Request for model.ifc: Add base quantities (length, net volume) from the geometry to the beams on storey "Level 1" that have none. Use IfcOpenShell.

First a look at what the model holds.

```python
import ifcopenshell
import ifcopenshell.util.element
import ifcopenshell.util.unit

model = ifcopenshell.open("model.ifc")
print(model.schema)
for unit_type in ("LENGTHUNIT", "AREAUNIT", "VOLUMEUNIT"):
    print(unit_type, ifcopenshell.util.unit.calculate_unit_scale(model, unit_type))
storey = next(s for s in model.by_type("IfcBuildingStorey") if s.Name == "Level 1")
beams = [e for e in ifcopenshell.util.element.get_decomposition(storey) if e.is_a("IfcBeam")]
for e in sorted(beams, key=lambda e: e.id()):
    print(e.id(), e.is_a(), e.Name, list(ifcopenshell.util.element.get_psets(e, qtos_only=True)), sep=" | ")
```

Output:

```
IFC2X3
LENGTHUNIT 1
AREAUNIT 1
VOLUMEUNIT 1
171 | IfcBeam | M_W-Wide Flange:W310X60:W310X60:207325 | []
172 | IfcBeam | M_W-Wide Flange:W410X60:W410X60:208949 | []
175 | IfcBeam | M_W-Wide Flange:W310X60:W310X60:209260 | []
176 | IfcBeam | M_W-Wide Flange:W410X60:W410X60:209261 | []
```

```python
import ifcopenshell
import ifcopenshell.api.pset
import ifcopenshell.geom
import ifcopenshell.util.element
import ifcopenshell.util.shape
import ifcopenshell.util.unit

model = ifcopenshell.open("model.ifc")
unit_scale = ifcopenshell.util.unit.calculate_unit_scale(model)
volume_scale = ifcopenshell.util.unit.calculate_unit_scale(model, "VOLUMEUNIT")
settings = ifcopenshell.geom.settings()

storey = next(s for s in model.by_type("IfcBuildingStorey") if s.Name == "Level 1")
beams = [e for e in ifcopenshell.util.element.get_decomposition(storey) if e.is_a("IfcBeam")]

for e in sorted(beams, key=lambda e: e.id()):
    if ifcopenshell.util.element.get_psets(e, qtos_only=True, should_inherit=False):
        continue
    # Geometry comes back in metres, in the element's own axes.
    shape = ifcopenshell.geom.create_shape(settings, e)
    values = {
        "Length": ifcopenshell.util.shape.get_max_xyz(shape.geometry) / unit_scale,
        "NetVolume": ifcopenshell.util.shape.get_volume(shape.geometry) / volume_scale,
    }
    qto = ifcopenshell.api.pset.add_qto(model, product=e, name="BaseQuantities")
    ifcopenshell.api.pset.edit_qto(model, qto=qto, properties=values)
    print(e.id(), {k: round(v, 3) for k, v in values.items()})

model.write("model_updated.ifc")
```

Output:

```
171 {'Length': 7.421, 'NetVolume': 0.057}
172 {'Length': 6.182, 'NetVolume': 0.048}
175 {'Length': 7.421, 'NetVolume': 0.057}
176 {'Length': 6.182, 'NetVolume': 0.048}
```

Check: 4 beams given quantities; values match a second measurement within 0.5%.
